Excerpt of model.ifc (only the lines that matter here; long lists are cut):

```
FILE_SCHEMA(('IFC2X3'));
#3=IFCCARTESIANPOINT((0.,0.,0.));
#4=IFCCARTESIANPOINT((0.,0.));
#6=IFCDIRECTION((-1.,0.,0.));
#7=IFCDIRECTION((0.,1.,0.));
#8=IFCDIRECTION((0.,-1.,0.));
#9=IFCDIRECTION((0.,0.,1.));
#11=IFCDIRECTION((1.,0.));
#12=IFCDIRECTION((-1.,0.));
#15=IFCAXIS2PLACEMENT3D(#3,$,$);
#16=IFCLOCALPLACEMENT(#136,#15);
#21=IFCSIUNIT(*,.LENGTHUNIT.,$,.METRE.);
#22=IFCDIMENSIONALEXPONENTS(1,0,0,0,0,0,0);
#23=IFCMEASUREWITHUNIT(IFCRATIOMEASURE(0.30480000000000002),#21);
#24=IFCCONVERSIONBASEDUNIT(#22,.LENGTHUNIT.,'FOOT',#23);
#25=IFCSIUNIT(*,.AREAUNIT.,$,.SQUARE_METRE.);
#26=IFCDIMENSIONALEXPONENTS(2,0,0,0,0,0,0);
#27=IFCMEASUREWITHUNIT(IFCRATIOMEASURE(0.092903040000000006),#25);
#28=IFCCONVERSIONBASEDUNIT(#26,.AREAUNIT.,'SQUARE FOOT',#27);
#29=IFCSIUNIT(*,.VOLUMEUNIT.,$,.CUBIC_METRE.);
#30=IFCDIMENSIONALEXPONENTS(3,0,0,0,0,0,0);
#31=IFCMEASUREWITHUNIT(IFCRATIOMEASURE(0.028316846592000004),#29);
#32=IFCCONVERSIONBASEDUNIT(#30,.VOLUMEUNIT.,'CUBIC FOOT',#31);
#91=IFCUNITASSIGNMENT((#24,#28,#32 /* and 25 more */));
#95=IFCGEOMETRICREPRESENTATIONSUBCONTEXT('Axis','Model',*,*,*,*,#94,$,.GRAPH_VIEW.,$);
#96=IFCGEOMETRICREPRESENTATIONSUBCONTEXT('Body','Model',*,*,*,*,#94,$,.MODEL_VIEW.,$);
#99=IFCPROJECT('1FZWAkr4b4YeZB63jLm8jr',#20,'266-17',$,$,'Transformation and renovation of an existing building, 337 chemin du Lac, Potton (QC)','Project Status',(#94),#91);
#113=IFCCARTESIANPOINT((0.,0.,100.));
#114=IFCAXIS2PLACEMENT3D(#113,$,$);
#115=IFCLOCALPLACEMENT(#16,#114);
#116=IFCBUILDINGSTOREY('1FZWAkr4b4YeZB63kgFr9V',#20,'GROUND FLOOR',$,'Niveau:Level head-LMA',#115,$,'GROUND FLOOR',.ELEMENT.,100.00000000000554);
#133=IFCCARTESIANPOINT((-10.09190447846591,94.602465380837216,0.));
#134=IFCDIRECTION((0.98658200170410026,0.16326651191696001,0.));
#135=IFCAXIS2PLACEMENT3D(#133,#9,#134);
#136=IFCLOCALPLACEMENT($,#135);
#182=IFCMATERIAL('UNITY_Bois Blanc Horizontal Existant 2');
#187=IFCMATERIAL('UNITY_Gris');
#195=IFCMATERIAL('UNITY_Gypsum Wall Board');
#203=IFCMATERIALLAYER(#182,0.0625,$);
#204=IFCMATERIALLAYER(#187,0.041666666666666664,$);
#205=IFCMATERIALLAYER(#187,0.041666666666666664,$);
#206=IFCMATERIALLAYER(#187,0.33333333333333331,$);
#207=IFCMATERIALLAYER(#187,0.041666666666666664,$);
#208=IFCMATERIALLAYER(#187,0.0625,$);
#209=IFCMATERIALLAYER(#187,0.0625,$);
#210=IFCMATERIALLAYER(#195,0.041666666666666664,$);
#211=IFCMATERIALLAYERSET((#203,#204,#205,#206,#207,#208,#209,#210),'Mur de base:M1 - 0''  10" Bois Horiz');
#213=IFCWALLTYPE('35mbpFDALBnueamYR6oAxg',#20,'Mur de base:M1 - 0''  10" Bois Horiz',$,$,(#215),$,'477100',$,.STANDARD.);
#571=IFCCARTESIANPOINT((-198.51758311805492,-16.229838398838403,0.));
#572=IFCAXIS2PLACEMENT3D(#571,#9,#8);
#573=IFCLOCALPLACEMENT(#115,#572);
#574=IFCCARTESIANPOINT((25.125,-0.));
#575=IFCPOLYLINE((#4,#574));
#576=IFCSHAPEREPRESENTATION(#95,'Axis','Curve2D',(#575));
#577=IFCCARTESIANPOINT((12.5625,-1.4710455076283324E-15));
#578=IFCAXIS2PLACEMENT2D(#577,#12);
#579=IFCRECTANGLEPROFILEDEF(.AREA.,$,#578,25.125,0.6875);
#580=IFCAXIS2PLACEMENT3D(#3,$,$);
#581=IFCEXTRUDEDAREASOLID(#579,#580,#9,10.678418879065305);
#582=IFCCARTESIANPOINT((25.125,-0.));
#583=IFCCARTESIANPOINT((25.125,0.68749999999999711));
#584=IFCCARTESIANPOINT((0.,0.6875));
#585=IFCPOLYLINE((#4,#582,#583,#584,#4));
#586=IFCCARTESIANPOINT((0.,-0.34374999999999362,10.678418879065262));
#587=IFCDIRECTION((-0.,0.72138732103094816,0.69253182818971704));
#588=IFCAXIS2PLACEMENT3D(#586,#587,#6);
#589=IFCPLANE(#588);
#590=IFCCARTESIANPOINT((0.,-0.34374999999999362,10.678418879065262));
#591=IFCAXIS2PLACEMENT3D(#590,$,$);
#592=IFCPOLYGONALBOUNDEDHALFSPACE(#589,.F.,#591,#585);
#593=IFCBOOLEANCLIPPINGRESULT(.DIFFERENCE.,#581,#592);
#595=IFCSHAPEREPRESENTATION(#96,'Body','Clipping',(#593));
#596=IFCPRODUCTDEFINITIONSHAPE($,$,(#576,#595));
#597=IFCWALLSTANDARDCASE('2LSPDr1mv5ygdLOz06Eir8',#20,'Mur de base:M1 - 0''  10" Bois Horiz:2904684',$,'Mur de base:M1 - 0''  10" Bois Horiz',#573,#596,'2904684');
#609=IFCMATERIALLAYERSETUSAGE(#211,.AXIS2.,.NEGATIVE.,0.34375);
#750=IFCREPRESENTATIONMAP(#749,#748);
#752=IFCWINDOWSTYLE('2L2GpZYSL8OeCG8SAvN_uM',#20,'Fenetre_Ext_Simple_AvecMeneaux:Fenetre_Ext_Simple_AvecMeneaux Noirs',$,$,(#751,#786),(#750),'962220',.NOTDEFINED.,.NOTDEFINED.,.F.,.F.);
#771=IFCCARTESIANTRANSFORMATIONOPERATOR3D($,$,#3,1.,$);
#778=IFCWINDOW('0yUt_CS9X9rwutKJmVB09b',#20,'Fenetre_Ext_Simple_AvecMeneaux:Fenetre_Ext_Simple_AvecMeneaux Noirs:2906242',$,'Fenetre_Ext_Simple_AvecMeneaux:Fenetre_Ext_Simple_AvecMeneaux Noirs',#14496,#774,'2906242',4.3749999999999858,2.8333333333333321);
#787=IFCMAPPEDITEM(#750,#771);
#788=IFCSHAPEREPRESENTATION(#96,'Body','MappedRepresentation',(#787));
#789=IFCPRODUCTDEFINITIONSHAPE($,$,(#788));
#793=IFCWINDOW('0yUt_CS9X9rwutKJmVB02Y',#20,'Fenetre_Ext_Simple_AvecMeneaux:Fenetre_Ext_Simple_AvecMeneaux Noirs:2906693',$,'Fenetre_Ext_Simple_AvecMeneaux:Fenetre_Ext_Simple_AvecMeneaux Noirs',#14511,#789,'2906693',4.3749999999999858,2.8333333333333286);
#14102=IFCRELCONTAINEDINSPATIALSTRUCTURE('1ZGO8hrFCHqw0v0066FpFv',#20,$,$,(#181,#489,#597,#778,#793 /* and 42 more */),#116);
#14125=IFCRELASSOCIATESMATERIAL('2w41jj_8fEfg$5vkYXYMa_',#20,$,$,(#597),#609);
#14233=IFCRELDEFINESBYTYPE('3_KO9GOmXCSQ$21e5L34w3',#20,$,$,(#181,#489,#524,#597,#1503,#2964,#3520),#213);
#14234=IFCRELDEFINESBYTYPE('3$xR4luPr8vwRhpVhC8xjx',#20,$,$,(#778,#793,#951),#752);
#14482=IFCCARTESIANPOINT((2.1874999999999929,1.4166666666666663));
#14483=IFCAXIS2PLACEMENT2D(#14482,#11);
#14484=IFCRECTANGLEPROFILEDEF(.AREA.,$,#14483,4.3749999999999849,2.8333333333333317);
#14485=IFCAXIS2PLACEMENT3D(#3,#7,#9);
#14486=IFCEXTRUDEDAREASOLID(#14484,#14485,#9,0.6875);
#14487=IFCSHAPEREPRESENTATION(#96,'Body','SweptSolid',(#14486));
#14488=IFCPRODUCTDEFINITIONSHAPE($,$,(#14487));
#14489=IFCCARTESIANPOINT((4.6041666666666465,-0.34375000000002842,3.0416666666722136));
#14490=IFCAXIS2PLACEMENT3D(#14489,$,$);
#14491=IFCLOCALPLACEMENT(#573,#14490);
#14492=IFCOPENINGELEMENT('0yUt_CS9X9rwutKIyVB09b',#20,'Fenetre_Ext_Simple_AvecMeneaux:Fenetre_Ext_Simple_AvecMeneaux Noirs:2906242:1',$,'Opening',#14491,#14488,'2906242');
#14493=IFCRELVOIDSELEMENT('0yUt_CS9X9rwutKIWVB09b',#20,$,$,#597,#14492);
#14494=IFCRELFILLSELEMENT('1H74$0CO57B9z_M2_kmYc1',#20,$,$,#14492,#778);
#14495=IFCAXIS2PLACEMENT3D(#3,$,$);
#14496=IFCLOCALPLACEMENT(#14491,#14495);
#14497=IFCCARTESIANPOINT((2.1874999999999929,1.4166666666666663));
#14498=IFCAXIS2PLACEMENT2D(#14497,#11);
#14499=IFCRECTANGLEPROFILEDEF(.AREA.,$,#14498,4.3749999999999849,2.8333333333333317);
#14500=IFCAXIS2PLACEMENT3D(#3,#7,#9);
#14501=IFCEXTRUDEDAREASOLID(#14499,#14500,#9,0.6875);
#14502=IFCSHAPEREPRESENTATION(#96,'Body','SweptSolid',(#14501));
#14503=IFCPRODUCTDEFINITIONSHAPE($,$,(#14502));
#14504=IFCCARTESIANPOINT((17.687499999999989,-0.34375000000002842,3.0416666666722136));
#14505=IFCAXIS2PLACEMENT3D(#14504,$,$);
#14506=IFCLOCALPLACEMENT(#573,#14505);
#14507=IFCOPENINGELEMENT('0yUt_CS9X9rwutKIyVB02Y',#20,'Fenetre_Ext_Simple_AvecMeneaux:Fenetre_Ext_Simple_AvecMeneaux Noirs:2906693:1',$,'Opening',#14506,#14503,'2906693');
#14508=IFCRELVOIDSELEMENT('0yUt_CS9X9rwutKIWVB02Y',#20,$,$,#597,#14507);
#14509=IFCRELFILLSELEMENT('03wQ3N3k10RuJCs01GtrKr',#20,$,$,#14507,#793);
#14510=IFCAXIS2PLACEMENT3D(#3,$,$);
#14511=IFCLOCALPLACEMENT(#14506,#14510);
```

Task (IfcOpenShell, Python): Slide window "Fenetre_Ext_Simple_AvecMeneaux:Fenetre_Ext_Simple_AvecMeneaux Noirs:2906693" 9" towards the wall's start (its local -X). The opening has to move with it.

```python
import ifcopenshell
import ifcopenshell.api.geometry
import ifcopenshell.util.placement
import ifcopenshell.util.unit

model = ifcopenshell.open("model.ifc")
unit_scale = ifcopenshell.util.unit.calculate_unit_scale(model)

window = model.by_guid("0yUt_CS9X9rwutKJmVB02Y")
opening = window.FillsVoids[0].RelatingOpeningElement
wall = opening.VoidsElements[0].RelatingBuildingElement

wall_matrix = ifcopenshell.util.placement.get_local_placement(wall.ObjectPlacement)
shift = wall_matrix[:3, 0] * -9 * 0.0254 / unit_scale
before = ifcopenshell.util.placement.get_local_placement(window.ObjectPlacement)[:3, 3].copy()

# The window is placed relative to its opening, so it follows when the opening moves.
matrix = ifcopenshell.util.placement.get_local_placement(opening.ObjectPlacement)
matrix[:3, 3] += shift
ifcopenshell.api.geometry.edit_object_placement(
    model, product=opening, matrix=matrix, is_si=False, should_transform_children=True
)

after = ifcopenshell.util.placement.get_local_placement(window.ObjectPlacement)[:3, 3]
print("window moved by", (after - before).round(3) + 0.0)

model.write("model_edited.ifc")
```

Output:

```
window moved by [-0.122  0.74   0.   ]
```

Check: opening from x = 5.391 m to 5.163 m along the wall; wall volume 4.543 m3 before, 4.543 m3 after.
